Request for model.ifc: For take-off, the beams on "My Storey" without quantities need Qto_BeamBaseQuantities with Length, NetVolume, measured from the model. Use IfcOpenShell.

First a look at what the model holds.

```python
import ifcopenshell
import ifcopenshell.util.element
import ifcopenshell.util.unit

model = ifcopenshell.open("model.ifc")
print(model.schema)
for unit_type in ("LENGTHUNIT", "AREAUNIT", "VOLUMEUNIT"):
    print(unit_type, ifcopenshell.util.unit.calculate_unit_scale(model, unit_type))
storey = next(s for s in model.by_type("IfcBuildingStorey") if s.Name == "My Storey")
beams = [e for e in ifcopenshell.util.element.get_decomposition(storey) if e.is_a("IfcBeam")]
for e in sorted(beams, key=lambda e: e.id()):
    print(e.id(), e.is_a(), e.Name, list(ifcopenshell.util.element.get_psets(e, qtos_only=True)), sep=" | ")
```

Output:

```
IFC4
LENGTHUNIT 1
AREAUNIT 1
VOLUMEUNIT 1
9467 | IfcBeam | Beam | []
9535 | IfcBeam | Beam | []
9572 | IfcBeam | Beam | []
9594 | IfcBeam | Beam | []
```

```python
import ifcopenshell
import ifcopenshell.api.pset
import ifcopenshell.geom
import ifcopenshell.util.element
import ifcopenshell.util.shape
import ifcopenshell.util.unit

model = ifcopenshell.open("model.ifc")
unit_scale = ifcopenshell.util.unit.calculate_unit_scale(model)
volume_scale = ifcopenshell.util.unit.calculate_unit_scale(model, "VOLUMEUNIT")
settings = ifcopenshell.geom.settings()

storey = next(s for s in model.by_type("IfcBuildingStorey") if s.Name == "My Storey")
beams = [e for e in ifcopenshell.util.element.get_decomposition(storey) if e.is_a("IfcBeam")]

for e in sorted(beams, key=lambda e: e.id()):
    if ifcopenshell.util.element.get_psets(e, qtos_only=True, should_inherit=False):
        continue
    # Geometry comes back in metres, in the element's own axes.
    shape = ifcopenshell.geom.create_shape(settings, e)
    values = {
        "Length": ifcopenshell.util.shape.get_max_xyz(shape.geometry) / unit_scale,
        "NetVolume": ifcopenshell.util.shape.get_volume(shape.geometry) / volume_scale,
    }
    qto = ifcopenshell.api.pset.add_qto(model, product=e, name="Qto_BeamBaseQuantities")
    ifcopenshell.api.pset.edit_qto(model, qto=qto, properties=values)
    print(e.id(), {k: round(v, 3) for k, v in values.items()})

model.write("model_updated.ifc")
```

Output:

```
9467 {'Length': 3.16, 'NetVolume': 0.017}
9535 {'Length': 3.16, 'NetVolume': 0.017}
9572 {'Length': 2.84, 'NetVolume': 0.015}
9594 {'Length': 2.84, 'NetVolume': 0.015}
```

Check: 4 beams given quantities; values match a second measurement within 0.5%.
